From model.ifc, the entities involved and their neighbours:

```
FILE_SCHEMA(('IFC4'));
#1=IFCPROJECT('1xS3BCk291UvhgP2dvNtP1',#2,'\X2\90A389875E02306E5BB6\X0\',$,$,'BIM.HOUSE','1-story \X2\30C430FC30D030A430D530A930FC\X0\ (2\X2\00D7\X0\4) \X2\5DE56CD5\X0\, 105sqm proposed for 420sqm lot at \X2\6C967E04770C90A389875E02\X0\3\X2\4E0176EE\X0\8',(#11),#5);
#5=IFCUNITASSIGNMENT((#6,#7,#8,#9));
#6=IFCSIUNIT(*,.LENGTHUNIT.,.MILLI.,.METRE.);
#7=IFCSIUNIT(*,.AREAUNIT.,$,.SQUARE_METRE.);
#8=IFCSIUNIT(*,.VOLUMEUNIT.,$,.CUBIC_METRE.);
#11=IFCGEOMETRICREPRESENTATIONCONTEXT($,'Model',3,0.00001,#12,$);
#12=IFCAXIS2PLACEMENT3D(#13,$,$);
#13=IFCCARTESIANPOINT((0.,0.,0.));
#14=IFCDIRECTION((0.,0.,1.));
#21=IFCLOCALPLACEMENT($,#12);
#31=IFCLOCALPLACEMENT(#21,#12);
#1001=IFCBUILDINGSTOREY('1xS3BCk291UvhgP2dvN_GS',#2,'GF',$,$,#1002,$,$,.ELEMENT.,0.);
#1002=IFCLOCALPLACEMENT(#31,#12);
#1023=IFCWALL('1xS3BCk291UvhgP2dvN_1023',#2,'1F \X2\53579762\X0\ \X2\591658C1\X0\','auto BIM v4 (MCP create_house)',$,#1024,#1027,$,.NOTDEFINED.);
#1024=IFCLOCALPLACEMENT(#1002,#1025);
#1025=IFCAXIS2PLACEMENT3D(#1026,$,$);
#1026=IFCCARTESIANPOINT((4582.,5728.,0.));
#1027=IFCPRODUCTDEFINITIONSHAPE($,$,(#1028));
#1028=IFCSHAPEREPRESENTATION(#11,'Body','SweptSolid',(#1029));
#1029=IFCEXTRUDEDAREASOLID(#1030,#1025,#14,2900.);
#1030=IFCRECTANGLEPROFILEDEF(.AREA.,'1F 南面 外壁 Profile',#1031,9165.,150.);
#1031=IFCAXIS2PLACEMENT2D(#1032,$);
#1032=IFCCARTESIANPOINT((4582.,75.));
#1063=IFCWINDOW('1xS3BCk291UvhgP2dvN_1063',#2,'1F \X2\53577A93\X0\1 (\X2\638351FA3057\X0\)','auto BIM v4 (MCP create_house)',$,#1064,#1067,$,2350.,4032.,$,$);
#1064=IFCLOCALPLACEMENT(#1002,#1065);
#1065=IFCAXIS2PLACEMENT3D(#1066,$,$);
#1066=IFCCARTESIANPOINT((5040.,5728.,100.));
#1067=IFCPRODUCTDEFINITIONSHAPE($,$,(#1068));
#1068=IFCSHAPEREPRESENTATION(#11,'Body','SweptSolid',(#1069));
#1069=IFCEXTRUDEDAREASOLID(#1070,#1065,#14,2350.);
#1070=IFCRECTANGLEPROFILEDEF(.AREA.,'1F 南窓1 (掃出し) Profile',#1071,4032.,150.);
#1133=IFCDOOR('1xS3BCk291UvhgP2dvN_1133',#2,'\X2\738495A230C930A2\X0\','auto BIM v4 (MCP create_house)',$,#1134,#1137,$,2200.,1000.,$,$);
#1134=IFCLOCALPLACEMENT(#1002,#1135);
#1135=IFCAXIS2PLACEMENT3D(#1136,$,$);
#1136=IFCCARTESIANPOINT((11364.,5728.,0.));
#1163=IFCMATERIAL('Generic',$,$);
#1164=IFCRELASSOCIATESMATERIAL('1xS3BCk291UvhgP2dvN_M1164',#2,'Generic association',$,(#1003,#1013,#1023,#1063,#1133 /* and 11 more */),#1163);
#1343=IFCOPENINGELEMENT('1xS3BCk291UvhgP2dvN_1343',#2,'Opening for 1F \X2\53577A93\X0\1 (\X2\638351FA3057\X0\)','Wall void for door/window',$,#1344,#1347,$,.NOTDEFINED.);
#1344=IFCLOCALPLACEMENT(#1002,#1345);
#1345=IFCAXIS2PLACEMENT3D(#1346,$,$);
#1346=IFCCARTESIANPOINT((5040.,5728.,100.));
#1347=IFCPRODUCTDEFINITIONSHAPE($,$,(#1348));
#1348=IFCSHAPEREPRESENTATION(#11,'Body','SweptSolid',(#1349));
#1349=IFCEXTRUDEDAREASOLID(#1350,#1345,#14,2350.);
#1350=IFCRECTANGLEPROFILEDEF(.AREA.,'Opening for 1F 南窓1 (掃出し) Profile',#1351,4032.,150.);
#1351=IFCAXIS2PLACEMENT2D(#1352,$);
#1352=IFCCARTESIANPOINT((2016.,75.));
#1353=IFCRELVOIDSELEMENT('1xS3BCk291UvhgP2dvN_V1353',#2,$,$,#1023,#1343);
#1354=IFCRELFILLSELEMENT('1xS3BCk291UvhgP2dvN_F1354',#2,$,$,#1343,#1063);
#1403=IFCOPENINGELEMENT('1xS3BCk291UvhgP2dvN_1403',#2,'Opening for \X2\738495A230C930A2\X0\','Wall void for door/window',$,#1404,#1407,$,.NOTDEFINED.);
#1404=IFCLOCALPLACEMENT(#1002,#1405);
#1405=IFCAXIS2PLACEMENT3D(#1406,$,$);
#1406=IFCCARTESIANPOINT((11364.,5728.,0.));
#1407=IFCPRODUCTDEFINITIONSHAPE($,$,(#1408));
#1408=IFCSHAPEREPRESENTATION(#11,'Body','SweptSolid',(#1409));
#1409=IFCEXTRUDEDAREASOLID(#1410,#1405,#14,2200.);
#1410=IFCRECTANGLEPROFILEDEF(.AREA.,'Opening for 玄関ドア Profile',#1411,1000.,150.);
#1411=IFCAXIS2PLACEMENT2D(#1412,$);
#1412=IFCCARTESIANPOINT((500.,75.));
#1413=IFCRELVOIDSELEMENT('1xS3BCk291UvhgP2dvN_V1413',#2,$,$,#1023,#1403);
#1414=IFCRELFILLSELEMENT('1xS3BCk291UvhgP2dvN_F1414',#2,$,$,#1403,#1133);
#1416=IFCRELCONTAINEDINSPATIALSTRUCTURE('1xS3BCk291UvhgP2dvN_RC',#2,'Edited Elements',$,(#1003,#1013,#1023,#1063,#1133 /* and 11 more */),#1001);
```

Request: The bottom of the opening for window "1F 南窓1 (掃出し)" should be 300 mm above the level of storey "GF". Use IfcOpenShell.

```python
import numpy as np
import ifcopenshell
import ifcopenshell.api.geometry
import ifcopenshell.geom
import ifcopenshell.util.element
import ifcopenshell.util.placement
import ifcopenshell.util.shape
import ifcopenshell.util.unit

model = ifcopenshell.open("model.ifc")
unit_scale = ifcopenshell.util.unit.calculate_unit_scale(model)

window = model.by_guid("1xS3BCk291UvhgP2dvN_1063")
opening = window.FillsVoids[0].RelatingOpeningElement
storey = ifcopenshell.util.element.get_container(window, ifc_class="IfcBuildingStorey")
level = ifcopenshell.util.placement.get_local_placement(storey.ObjectPlacement)[2, 3]

# The opening's origin need not be at the sill, so measure its lowest point.
shape = ifcopenshell.geom.create_shape(ifcopenshell.geom.settings(), opening)
bottom = ifcopenshell.util.shape.get_shape_bottom_elevation(shape, shape.geometry) / unit_scale
dz = level + 0.3 / unit_scale - bottom

shift = np.array([0.0, 0.0, dz])
# The window is not placed relative to its opening, so move both.
for product in (opening, window):
    matrix = ifcopenshell.util.placement.get_local_placement(product.ObjectPlacement)
    matrix[:3, 3] += shift
    ifcopenshell.api.geometry.edit_object_placement(model, product=product, matrix=matrix, is_si=False)

print(f"moved by {dz * unit_scale:+.3f} m")

model.write("model_rev.ifc")
```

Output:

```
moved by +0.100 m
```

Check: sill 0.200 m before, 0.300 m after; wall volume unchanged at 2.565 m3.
